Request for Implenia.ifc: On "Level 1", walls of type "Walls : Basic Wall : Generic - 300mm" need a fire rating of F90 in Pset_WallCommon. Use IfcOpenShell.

First a look at what the model holds.

```python
import ifcopenshell
import ifcopenshell.util.element

model = ifcopenshell.open("Implenia.ifc")
print(model.schema)
storey = next(s for s in model.by_type("IfcBuildingStorey") if s.Name == "Level 1")
walls = [e for e in ifcopenshell.util.element.get_decomposition(storey) if e.is_a("IfcWall")]
seen = {}
for e in walls:
    element_type = ifcopenshell.util.element.get_type(e)
    key = (element_type.Name if element_type != e and element_type else None, ifcopenshell.util.element.get_pset(e, "Pset_WallCommon", "FireRating"))
    seen[key] = seen.get(key, 0) + 1
for (name, value), count in sorted(seen.items(), key=str):
    print(count, "x", name, "|", value)
```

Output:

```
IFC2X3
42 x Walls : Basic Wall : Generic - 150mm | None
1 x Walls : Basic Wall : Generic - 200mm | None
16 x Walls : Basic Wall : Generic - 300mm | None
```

```python
import ifcopenshell
import ifcopenshell.api.pset
import ifcopenshell.util.element

model = ifcopenshell.open("Implenia.ifc")

storey = next(s for s in model.by_type("IfcBuildingStorey") if s.Name == "Level 1")
walls = [e for e in ifcopenshell.util.element.get_decomposition(storey) if e.is_a("IfcWall")]

count = 0
for e in walls:
    element_type = ifcopenshell.util.element.get_type(e)
    if element_type in (None, e) or element_type.Name != "Walls : Basic Wall : Generic - 300mm":
        continue
    # add_pset returns the element's existing set when there is one.
    pset = ifcopenshell.api.pset.add_pset(model, product=e, name="Pset_WallCommon")
    ifcopenshell.api.pset.edit_pset(model, pset=pset, properties={"FireRating": "F90"})
    count += 1

print(count, "walls updated")

model.write("Implenia_updated.ifc")
```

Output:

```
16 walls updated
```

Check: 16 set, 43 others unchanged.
